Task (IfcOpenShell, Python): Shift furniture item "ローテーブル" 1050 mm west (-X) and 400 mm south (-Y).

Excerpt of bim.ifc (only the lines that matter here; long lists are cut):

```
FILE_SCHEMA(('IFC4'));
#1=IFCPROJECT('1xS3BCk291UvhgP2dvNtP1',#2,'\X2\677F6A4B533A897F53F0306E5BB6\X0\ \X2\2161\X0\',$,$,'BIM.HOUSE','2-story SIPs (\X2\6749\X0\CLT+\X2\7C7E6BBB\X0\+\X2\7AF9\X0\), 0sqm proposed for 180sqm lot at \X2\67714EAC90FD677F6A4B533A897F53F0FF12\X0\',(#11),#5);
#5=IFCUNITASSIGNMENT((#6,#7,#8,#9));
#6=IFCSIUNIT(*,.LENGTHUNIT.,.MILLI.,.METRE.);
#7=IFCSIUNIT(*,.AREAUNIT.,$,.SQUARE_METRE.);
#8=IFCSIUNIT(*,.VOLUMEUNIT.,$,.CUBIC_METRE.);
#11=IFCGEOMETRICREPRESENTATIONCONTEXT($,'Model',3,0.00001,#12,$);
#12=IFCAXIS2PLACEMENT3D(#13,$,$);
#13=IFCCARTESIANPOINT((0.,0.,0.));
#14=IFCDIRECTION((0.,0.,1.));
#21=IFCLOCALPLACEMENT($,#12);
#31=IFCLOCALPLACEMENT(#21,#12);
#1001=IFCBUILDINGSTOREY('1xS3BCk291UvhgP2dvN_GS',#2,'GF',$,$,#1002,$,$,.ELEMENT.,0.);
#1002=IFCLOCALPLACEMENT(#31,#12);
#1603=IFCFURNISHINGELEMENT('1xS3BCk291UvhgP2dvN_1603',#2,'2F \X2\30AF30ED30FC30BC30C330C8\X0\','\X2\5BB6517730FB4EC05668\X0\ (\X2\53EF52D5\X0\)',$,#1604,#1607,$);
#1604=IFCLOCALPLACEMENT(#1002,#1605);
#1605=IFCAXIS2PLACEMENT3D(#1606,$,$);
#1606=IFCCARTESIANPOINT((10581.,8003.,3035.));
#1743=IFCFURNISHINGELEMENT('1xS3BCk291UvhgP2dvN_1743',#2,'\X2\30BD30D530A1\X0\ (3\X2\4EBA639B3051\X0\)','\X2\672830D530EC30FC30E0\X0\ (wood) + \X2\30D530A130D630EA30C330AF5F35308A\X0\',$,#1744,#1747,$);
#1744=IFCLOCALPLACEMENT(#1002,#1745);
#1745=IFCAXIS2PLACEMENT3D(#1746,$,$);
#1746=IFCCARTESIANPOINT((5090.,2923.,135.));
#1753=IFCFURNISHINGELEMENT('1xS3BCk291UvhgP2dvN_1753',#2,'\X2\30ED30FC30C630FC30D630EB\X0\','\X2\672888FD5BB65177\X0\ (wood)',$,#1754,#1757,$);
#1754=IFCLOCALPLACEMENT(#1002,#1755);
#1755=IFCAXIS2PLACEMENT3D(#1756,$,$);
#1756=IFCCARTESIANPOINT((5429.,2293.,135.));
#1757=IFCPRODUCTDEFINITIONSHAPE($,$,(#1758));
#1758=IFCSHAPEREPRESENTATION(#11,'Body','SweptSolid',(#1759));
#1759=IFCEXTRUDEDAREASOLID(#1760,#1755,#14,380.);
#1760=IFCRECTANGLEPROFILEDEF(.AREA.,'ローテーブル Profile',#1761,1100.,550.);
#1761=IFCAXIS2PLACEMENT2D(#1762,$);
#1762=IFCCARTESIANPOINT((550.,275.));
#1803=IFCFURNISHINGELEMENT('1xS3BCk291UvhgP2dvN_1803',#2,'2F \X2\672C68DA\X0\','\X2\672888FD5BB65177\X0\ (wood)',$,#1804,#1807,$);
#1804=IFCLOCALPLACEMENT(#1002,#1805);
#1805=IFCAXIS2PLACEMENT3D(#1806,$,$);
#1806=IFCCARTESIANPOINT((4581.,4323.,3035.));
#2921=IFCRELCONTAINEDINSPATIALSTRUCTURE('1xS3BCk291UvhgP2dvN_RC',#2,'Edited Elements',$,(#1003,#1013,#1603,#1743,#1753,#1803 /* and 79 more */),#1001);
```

```python
import ifcopenshell
import ifcopenshell.api.geometry
import ifcopenshell.util.placement

model = ifcopenshell.open("bim.ifc")

item = model.by_guid("1xS3BCk291UvhgP2dvN_1753")
matrix = ifcopenshell.util.placement.get_local_placement(item.ObjectPlacement)
matrix[0, 3] -= 1050.0
matrix[1, 3] -= 400.0
ifcopenshell.api.geometry.edit_object_placement(model, product=item, matrix=matrix, is_si=False)

print(ifcopenshell.util.placement.get_local_placement(item.ObjectPlacement).round(3) + 0.0)

model.write("bim_updated.ifc")
```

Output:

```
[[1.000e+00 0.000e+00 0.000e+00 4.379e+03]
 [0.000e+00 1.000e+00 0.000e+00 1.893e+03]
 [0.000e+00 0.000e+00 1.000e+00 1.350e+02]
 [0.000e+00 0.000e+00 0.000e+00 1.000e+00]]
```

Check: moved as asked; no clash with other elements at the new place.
